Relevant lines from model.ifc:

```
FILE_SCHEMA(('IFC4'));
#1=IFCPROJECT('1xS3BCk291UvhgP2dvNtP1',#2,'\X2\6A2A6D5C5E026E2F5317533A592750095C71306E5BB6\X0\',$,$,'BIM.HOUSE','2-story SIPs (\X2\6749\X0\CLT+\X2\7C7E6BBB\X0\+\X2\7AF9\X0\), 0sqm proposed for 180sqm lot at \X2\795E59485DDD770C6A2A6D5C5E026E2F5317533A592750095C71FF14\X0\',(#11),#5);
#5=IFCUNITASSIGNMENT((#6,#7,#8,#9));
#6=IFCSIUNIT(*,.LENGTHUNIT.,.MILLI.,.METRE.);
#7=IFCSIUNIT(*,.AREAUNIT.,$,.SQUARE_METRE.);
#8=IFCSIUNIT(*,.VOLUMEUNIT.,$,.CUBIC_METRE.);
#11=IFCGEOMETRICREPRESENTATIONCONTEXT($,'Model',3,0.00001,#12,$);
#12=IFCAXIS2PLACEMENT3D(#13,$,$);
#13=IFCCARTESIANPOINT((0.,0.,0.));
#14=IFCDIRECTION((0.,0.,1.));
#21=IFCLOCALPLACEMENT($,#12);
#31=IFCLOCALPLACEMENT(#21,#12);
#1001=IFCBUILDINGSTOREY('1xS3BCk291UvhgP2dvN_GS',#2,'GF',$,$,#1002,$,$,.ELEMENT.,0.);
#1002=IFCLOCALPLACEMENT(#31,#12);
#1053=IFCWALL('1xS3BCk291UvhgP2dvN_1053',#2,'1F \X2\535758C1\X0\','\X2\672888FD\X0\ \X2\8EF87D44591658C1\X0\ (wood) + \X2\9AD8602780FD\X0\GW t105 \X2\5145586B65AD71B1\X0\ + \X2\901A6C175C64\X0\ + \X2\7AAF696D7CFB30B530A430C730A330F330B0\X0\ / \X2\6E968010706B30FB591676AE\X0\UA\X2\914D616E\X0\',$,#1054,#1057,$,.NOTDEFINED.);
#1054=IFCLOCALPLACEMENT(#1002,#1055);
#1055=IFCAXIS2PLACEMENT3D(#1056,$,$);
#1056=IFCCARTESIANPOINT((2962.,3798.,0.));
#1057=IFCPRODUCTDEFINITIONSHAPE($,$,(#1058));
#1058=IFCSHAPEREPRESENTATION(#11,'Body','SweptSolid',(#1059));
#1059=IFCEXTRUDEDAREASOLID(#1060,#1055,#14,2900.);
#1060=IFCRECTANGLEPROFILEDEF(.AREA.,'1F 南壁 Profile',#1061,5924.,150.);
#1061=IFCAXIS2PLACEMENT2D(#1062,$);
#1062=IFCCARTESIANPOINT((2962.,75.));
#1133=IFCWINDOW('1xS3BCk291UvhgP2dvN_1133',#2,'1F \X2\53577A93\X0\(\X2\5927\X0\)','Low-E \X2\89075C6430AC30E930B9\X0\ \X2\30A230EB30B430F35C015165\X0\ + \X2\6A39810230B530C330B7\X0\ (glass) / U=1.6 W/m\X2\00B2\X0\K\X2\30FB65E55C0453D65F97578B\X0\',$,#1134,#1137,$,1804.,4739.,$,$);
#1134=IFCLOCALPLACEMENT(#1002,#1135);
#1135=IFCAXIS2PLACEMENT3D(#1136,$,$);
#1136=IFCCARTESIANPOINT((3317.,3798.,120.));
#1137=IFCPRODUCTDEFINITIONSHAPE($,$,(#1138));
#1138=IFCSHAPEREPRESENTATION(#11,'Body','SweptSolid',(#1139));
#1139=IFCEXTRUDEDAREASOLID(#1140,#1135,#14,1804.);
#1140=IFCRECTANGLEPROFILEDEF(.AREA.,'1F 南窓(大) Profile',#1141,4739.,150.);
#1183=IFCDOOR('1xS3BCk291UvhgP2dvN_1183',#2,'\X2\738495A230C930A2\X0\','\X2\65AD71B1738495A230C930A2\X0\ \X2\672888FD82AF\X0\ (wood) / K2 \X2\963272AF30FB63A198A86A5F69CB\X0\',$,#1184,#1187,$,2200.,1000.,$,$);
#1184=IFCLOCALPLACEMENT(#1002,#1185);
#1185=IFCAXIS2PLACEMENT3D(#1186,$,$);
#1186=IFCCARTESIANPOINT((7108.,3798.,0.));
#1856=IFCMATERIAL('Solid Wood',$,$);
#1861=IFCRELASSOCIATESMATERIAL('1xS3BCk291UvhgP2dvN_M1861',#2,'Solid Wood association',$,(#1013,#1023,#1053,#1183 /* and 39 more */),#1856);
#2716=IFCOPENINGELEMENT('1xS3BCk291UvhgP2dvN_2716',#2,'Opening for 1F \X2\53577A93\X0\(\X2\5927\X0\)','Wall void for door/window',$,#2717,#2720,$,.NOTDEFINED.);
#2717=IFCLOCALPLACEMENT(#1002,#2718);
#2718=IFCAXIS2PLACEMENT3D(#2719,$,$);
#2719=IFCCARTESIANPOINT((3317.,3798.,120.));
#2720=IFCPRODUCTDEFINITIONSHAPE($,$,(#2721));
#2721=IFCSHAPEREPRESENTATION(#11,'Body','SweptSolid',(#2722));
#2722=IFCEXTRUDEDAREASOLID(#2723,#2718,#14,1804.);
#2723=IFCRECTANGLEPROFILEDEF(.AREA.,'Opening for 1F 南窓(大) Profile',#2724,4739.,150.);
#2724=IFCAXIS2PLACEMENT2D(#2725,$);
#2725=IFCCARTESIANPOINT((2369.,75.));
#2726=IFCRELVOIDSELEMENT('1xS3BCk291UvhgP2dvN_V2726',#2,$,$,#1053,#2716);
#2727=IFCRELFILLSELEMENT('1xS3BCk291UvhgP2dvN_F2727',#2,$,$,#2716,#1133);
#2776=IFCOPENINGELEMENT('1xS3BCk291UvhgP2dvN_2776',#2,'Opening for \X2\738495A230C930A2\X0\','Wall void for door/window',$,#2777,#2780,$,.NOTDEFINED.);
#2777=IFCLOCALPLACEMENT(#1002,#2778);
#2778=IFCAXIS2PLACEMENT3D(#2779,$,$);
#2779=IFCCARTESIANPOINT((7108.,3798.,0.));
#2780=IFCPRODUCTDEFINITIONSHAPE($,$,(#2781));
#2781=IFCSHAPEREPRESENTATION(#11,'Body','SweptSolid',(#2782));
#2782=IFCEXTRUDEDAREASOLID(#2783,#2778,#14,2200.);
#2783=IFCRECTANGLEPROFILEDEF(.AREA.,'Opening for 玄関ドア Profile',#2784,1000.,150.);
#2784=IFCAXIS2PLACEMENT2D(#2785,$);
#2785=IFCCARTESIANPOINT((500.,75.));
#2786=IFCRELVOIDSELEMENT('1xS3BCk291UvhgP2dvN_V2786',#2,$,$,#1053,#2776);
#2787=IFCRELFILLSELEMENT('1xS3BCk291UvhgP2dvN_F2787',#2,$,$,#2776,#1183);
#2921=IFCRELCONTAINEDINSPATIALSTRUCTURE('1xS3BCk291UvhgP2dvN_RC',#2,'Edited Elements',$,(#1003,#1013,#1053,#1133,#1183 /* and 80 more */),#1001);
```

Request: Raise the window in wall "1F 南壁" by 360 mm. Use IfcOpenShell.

```python
import numpy as np
import ifcopenshell
import ifcopenshell.api.geometry
import ifcopenshell.util.placement
import ifcopenshell.util.unit

model = ifcopenshell.open("model.ifc")
unit_scale = ifcopenshell.util.unit.calculate_unit_scale(model)

window = model.by_id(1133)
opening = window.FillsVoids[0].RelatingOpeningElement
dz = 0.36 / unit_scale

shift = np.array([0.0, 0.0, dz])
# The window is not placed relative to its opening, so move both.
for product in (opening, window):
    matrix = ifcopenshell.util.placement.get_local_placement(product.ObjectPlacement)
    matrix[:3, 3] += shift
    ifcopenshell.api.geometry.edit_object_placement(model, product=product, matrix=matrix, is_si=False)

print(f"moved by {dz * unit_scale:+.3f} m")

model.write("model_edited.ifc")
```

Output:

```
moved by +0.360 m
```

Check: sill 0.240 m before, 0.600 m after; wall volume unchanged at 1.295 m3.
